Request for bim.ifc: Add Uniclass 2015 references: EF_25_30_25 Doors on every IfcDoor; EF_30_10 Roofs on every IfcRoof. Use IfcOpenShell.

First a look at what the model holds.

```python
import ifcopenshell

model = ifcopenshell.open("bim.ifc")
print(model.schema)
print("classifications:", [c.Name for c in model.by_type("IfcClassification")])
for ifc_class in ("IfcDoor", "IfcRoof", "IfcStair", "IfcWall", "IfcWindow"):
    print(ifc_class, len(model.by_type(ifc_class)))
```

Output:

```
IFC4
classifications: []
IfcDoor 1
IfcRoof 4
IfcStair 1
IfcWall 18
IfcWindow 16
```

```python
import ifcopenshell
import ifcopenshell.api.classification

model = ifcopenshell.open("bim.ifc")

system = ifcopenshell.api.classification.add_classification(model, classification="Uniclass 2015")

codes = {
    "IfcDoor": ("EF_25_30_25", "Doors"),
    "IfcRoof": ("EF_30_10", "Roofs"),
}
for ifc_class, (code, name) in codes.items():
    products = model.by_type(ifc_class)
    ifcopenshell.api.classification.add_reference(
        model, products=products, classification=system, identification=code, name=name
    )
    print(code, len(products))

model.write("bim_v2.ifc")
```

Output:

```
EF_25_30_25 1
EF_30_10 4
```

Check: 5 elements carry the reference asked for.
